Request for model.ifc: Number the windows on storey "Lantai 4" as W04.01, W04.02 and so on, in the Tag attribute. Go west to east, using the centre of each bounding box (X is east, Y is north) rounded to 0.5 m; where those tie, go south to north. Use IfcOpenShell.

First a look at what the model holds.

```python
import ifcopenshell
import ifcopenshell.util.element
import ifcopenshell.util.placement

model = ifcopenshell.open("model.ifc")
print(model.schema)
storey = next(s for s in model.by_type("IfcBuildingStorey") if s.Name == "Lantai 4")
windows = [e for e in ifcopenshell.util.element.get_decomposition(storey) if e.is_a("IfcWindow")]
for e in sorted(windows, key=lambda e: e.id()):
    origin = ifcopenshell.util.placement.get_local_placement(e.ObjectPlacement)[:3, 3]
    print(e.id(), e.Tag, e.Name, origin.round(2) + 0.0, sep=" | ")
```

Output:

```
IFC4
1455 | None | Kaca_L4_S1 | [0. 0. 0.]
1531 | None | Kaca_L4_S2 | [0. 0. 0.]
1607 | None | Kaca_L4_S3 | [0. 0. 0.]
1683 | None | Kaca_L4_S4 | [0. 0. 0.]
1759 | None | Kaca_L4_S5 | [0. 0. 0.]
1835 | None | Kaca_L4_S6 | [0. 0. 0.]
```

```python
import ifcopenshell
import ifcopenshell.geom
import ifcopenshell.util.element
import ifcopenshell.util.shape

model = ifcopenshell.open("model.ifc")
settings = ifcopenshell.geom.settings()
settings.set("use-world-coords", True)


def centre(element):
    shape = ifcopenshell.geom.create_shape(settings, element)
    return ifcopenshell.util.shape.get_bbox_centroid(shape.geometry)


storey = next(s for s in model.by_type("IfcBuildingStorey") if s.Name == "Lantai 4")
windows = [e for e in ifcopenshell.util.element.get_decomposition(storey) if e.is_a("IfcWindow")]

# Insertion points can sit at a corner or the storey origin, so sort by the geometry (in metres).
centres = {e: centre(e) for e in windows}
windows.sort(key=lambda e: (round(centres[e][0] / 0.5), centres[e][1]))

for i, e in enumerate(windows, start=1):
    number = f"W04.{i:02d}"
    e.Tag = number
    print(e.id(), number)

model.write("model_updated.ifc")
```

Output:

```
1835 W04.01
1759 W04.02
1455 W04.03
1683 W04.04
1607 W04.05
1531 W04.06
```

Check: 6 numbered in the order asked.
